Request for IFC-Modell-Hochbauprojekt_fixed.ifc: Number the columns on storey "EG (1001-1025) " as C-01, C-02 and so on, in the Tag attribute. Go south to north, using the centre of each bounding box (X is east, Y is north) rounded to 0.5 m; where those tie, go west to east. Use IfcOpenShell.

First a look at what the model holds.

```python
import ifcopenshell
import ifcopenshell.util.element
import ifcopenshell.util.placement

model = ifcopenshell.open("IFC-Modell-Hochbauprojekt_fixed.ifc")
print(model.schema)
storey = next(s for s in model.by_type("IfcBuildingStorey") if s.Name == "EG (1001-1025) ")
columns = [e for e in ifcopenshell.util.element.get_decomposition(storey) if e.is_a("IfcColumn")]
for e in sorted(columns, key=lambda e: e.id()):
    origin = ifcopenshell.util.placement.get_local_placement(e.ObjectPlacement)[:3, 3]
    print(e.id(), e.Tag, e.Name, origin.round(2) + 0.0, sep=" | ")
```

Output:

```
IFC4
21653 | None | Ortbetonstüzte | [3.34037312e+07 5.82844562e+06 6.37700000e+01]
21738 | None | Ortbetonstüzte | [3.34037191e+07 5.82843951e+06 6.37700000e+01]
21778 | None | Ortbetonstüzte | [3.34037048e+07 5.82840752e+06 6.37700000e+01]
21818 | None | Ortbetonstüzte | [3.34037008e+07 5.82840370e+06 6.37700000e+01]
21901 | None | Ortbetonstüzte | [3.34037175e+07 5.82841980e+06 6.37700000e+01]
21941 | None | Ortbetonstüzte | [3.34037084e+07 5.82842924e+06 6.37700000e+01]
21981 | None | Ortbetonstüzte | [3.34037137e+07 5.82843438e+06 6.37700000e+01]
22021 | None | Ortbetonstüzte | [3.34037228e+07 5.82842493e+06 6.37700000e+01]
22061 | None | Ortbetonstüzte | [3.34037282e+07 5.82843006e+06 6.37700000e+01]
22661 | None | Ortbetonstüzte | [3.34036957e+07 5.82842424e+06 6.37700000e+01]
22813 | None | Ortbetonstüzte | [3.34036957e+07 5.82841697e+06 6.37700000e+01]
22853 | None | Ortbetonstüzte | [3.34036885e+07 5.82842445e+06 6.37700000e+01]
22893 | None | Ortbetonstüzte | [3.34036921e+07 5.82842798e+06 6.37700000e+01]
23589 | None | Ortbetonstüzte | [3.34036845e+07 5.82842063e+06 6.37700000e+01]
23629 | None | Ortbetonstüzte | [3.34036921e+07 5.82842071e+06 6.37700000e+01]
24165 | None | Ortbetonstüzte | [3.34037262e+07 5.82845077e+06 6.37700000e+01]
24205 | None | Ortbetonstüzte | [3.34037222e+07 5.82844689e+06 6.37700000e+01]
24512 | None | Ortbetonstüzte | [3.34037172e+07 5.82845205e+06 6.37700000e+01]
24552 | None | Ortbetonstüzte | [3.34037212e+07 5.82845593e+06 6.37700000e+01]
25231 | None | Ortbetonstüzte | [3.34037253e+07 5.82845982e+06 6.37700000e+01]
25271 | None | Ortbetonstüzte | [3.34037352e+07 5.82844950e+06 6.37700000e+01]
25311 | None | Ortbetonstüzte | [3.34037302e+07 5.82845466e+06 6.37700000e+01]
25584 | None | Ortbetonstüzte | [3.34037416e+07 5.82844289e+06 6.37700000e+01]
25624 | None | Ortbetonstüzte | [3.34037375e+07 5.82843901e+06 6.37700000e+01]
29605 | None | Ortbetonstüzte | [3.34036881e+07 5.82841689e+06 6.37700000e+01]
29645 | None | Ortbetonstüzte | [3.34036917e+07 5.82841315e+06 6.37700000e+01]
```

```python
import ifcopenshell
import ifcopenshell.geom
import ifcopenshell.util.element
import ifcopenshell.util.shape

model = ifcopenshell.open("IFC-Modell-Hochbauprojekt_fixed.ifc")
settings = ifcopenshell.geom.settings()
settings.set("use-world-coords", True)


def centre(element):
    shape = ifcopenshell.geom.create_shape(settings, element)
    return ifcopenshell.util.shape.get_bbox_centroid(shape.geometry)


storey = next(s for s in model.by_type("IfcBuildingStorey") if s.Name == "EG (1001-1025) ")
columns = [e for e in ifcopenshell.util.element.get_decomposition(storey) if e.is_a("IfcColumn")]

# Insertion points can sit at a corner or the storey origin, so sort by the geometry (in metres).
centres = {e: centre(e) for e in columns}
columns.sort(key=lambda e: (round(centres[e][1] / 0.5), centres[e][0]))

for i, e in enumerate(columns, start=1):
    number = f"C-{i:02d}"
    e.Tag = number
    print(e.id(), number)

model.write("IFC-Modell-Hochbauprojekt_fixed_edited.ifc")
```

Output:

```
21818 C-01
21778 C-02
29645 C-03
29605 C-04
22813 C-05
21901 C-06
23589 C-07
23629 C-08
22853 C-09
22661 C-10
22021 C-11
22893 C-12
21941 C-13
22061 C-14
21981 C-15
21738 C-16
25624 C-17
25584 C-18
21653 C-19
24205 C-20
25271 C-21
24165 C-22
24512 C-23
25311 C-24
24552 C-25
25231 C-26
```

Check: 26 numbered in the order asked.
